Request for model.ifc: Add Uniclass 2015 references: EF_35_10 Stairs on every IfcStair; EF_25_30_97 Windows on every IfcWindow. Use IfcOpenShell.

First a look at what the model holds.

```python
import ifcopenshell

model = ifcopenshell.open("model.ifc")
print(model.schema)
print("classifications:", [c.Name for c in model.by_type("IfcClassification")])
for ifc_class in ("IfcDoor", "IfcRoof", "IfcStair", "IfcWall", "IfcWindow"):
    print(ifc_class, len(model.by_type(ifc_class)))
```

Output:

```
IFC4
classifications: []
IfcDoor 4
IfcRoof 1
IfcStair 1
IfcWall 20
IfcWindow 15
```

```python
import ifcopenshell
import ifcopenshell.api.classification

model = ifcopenshell.open("model.ifc")

system = ifcopenshell.api.classification.add_classification(model, classification="Uniclass 2015")

codes = {
    "IfcStair": ("EF_35_10", "Stairs"),
    "IfcWindow": ("EF_25_30_97", "Windows"),
}
for ifc_class, (code, name) in codes.items():
    products = model.by_type(ifc_class)
    ifcopenshell.api.classification.add_reference(
        model, products=products, classification=system, identification=code, name=name
    )
    print(code, len(products))

model.write("model_updated.ifc")
```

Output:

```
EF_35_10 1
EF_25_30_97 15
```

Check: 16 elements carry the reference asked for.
